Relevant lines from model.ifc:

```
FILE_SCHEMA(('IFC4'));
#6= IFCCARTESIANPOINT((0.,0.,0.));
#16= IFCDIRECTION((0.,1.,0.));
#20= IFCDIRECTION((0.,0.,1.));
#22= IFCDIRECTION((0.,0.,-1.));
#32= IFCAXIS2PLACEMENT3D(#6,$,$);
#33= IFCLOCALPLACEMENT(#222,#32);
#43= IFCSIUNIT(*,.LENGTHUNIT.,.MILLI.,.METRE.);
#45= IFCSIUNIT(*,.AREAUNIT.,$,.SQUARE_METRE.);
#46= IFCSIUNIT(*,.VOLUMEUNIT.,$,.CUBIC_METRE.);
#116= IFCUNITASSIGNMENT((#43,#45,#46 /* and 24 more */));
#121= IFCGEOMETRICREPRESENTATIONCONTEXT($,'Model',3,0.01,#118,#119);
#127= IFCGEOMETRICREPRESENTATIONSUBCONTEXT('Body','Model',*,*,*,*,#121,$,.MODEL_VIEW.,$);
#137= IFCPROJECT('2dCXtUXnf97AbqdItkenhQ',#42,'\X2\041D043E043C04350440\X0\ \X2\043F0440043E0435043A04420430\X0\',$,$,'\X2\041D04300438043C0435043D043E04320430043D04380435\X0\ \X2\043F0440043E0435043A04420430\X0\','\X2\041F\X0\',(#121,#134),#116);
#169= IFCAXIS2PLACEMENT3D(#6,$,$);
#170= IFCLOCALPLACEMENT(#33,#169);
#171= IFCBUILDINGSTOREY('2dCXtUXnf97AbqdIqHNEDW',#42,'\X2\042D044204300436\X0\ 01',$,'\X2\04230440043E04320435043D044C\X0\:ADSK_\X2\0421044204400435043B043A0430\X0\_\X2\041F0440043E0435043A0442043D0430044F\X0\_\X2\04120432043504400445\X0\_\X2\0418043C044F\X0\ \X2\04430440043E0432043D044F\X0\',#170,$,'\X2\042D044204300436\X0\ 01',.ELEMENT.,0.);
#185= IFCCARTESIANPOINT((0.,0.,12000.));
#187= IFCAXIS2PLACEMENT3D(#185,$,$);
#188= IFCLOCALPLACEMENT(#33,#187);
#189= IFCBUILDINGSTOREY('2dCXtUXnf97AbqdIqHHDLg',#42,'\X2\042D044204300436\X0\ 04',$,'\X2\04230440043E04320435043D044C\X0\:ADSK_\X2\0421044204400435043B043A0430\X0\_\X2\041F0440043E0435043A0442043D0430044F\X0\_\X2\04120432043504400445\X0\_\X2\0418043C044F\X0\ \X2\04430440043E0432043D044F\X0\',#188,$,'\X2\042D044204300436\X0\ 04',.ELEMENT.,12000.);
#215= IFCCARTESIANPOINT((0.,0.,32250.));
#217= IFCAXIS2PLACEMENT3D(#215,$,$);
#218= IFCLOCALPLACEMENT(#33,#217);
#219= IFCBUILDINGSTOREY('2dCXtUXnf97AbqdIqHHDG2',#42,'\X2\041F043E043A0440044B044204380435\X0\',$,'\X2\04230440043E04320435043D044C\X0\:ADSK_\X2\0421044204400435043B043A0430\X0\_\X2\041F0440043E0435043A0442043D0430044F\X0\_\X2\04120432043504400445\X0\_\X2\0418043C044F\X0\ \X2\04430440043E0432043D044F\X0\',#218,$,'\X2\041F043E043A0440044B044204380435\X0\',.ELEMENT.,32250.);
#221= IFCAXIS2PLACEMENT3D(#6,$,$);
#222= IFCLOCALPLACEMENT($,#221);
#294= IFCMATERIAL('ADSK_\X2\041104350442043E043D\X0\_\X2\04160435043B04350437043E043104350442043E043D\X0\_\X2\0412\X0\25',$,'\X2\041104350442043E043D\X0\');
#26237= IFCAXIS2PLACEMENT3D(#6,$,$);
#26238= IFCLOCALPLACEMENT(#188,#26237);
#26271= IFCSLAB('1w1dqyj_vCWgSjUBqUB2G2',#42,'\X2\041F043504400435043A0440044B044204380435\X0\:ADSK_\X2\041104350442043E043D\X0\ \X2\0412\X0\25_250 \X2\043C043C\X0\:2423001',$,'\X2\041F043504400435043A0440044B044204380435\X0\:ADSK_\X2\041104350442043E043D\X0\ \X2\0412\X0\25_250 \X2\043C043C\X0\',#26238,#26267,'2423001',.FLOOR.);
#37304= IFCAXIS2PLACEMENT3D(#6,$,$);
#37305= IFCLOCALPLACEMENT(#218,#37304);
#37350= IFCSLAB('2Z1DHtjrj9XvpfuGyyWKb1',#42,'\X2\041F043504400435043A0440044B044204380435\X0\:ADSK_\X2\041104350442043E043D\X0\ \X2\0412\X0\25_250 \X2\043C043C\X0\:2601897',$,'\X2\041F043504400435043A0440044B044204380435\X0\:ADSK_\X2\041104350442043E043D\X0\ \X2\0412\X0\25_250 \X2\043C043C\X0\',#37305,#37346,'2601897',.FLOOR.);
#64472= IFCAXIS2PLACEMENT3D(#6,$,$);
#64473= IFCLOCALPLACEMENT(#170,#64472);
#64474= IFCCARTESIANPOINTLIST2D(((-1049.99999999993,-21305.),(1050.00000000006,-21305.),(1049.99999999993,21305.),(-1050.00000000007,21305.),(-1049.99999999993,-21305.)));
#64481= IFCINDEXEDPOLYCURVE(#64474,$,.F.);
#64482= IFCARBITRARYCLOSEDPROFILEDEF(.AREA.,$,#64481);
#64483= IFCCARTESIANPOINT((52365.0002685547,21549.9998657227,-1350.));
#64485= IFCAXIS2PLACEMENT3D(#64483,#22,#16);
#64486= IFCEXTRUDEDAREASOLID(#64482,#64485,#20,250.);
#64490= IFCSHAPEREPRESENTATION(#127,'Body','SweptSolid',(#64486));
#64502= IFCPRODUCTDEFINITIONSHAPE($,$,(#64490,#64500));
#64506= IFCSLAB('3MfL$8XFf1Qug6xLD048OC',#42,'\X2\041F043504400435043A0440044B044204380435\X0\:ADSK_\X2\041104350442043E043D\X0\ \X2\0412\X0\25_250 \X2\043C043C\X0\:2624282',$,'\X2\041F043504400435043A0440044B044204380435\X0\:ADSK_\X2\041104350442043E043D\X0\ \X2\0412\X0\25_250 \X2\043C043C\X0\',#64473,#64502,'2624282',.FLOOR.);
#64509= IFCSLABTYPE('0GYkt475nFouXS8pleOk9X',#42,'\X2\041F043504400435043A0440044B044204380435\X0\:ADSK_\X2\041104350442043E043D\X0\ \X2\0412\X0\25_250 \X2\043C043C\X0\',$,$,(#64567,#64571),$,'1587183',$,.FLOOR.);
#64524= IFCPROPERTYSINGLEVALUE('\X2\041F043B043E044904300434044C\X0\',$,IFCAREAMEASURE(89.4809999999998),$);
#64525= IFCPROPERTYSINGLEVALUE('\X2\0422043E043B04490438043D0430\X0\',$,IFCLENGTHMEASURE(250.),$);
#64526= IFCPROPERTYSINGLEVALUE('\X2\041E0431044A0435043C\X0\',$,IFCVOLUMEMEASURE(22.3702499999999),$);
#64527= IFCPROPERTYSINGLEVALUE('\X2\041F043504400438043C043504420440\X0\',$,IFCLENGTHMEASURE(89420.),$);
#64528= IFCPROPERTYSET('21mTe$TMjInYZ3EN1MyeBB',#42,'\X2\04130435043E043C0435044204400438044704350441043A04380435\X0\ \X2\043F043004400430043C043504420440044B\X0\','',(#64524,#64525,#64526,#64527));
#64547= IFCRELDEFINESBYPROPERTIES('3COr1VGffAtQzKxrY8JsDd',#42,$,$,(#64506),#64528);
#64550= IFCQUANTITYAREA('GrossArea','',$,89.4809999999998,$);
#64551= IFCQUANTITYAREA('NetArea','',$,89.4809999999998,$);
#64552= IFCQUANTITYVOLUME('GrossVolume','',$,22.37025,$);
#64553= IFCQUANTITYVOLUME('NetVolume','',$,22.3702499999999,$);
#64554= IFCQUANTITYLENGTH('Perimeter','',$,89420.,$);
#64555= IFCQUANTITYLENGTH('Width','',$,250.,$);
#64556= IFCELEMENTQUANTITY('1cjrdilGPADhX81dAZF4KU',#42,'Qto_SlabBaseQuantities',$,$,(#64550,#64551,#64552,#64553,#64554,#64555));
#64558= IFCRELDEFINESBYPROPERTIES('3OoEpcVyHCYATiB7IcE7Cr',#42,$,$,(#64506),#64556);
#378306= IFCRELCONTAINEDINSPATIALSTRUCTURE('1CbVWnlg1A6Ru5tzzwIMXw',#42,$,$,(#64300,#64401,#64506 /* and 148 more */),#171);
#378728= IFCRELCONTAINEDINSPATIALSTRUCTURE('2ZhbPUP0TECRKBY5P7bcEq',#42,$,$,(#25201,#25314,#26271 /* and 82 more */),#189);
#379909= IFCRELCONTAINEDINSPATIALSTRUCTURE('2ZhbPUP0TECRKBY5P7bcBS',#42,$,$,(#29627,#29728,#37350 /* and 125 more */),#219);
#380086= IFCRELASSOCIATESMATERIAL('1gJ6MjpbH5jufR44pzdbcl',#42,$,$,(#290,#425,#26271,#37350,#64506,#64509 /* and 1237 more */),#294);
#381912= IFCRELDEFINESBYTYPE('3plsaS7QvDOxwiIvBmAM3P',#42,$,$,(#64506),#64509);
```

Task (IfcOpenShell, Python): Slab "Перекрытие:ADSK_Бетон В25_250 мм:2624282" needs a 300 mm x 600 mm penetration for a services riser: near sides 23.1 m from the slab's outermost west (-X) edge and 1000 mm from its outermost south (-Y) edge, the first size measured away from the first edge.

```python
import numpy as np
import ifcopenshell
import ifcopenshell.api.feature
import ifcopenshell.api.geometry
import ifcopenshell.api.pset
import ifcopenshell.api.root
import ifcopenshell.geom
import ifcopenshell.util.element
import ifcopenshell.util.placement
import ifcopenshell.util.representation
import ifcopenshell.util.shape
import ifcopenshell.util.unit

model = ifcopenshell.open("model.ifc")
unit_scale = ifcopenshell.util.unit.calculate_unit_scale(model)
area_scale = ifcopenshell.util.unit.calculate_unit_scale(model, "AREAUNIT")
volume_scale = ifcopenshell.util.unit.calculate_unit_scale(model, "VOLUMEUNIT")
settings = ifcopenshell.geom.settings()


def volume(element):
    """Net volume in cubic metres, openings subtracted."""
    shape = ifcopenshell.geom.create_shape(settings, element)
    return ifcopenshell.util.shape.get_volume(shape.geometry)


slab = model.by_id(64506)
before = volume(slab)

# Extent in the slab's own axes, in metres. The edges named are its -X and -Y sides.
slab_shape = ifcopenshell.geom.create_shape(settings, slab)
vertices = ifcopenshell.util.shape.get_vertices(slab_shape.geometry)
x_min, y_min, bottom = vertices.min(axis=0)
top = vertices[:, 2].max()

opening = ifcopenshell.api.root.create_entity(model, ifc_class="IfcOpeningElement", name="Services riser opening", predefined_type="OPENING")
context = ifcopenshell.util.representation.get_context(model, "Model", "Body", "MODEL_VIEW")
width, depth = 0.3, 0.6
outline = [(0.0, 0.0), (width, 0.0), (width, depth), (0.0, depth), (0.0, 0.0)]
# Overshoot both faces by 50 mm so the cut is clean.
shape = ifcopenshell.api.geometry.add_slab_representation(
    model, context=context, depth=top - bottom + 0.1, polyline=outline
)
ifcopenshell.api.geometry.assign_representation(model, product=opening, representation=shape)

matrix = ifcopenshell.util.placement.get_local_placement(slab.ObjectPlacement)
matrix[:, 3] = matrix @ np.append(np.array([x_min + 23.1, y_min + 1, bottom - 0.05]) / unit_scale, 1.0)
ifcopenshell.api.geometry.edit_object_placement(model, product=opening, matrix=matrix, is_si=False)
ifcopenshell.api.feature.add_feature(model, feature=opening, element=slab)

after = volume(slab)

# Update the slab's stored quantities.
pset = model.by_id(ifcopenshell.util.element.get_pset(slab, "Геометрические параметры", should_inherit=False)["id"])
ifcopenshell.api.pset.edit_pset(model, pset=pset, properties={
    "Площадь": model.create_entity("IfcAreaMeasure", after / (top - bottom) / area_scale),
    "Объем": model.create_entity("IfcVolumeMeasure", after / volume_scale),
})
qto = model.by_id(ifcopenshell.util.element.get_pset(slab, "Qto_SlabBaseQuantities", should_inherit=False)["id"])
ifcopenshell.api.pset.edit_qto(model, qto=qto, properties={
    "NetArea": after / (top - bottom) / area_scale,
    "NetVolume": after / volume_scale,
})

print(f"slab volume {before:.3f} -> {after:.3f} m3")

model.write("model-out.ifc")
```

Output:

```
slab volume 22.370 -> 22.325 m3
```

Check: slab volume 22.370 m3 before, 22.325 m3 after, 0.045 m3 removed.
